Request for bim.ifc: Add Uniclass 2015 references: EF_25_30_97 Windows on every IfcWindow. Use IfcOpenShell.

First a look at what the model holds.

```python
import ifcopenshell

model = ifcopenshell.open("bim.ifc")
print(model.schema)
print("classifications:", [c.Name for c in model.by_type("IfcClassification")])
for ifc_class in ("IfcDoor", "IfcRoof", "IfcStair", "IfcWall", "IfcWindow"):
    print(ifc_class, len(model.by_type(ifc_class)))
```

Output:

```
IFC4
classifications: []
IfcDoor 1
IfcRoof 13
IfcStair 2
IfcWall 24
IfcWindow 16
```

```python
import ifcopenshell
import ifcopenshell.api.classification

model = ifcopenshell.open("bim.ifc")

system = ifcopenshell.api.classification.add_classification(model, classification="Uniclass 2015")

codes = {
    "IfcWindow": ("EF_25_30_97", "Windows"),
}
for ifc_class, (code, name) in codes.items():
    products = model.by_type(ifc_class)
    ifcopenshell.api.classification.add_reference(
        model, products=products, classification=system, identification=code, name=name
    )
    print(code, len(products))

model.write("bim_v2.ifc")
```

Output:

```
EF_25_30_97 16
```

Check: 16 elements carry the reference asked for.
